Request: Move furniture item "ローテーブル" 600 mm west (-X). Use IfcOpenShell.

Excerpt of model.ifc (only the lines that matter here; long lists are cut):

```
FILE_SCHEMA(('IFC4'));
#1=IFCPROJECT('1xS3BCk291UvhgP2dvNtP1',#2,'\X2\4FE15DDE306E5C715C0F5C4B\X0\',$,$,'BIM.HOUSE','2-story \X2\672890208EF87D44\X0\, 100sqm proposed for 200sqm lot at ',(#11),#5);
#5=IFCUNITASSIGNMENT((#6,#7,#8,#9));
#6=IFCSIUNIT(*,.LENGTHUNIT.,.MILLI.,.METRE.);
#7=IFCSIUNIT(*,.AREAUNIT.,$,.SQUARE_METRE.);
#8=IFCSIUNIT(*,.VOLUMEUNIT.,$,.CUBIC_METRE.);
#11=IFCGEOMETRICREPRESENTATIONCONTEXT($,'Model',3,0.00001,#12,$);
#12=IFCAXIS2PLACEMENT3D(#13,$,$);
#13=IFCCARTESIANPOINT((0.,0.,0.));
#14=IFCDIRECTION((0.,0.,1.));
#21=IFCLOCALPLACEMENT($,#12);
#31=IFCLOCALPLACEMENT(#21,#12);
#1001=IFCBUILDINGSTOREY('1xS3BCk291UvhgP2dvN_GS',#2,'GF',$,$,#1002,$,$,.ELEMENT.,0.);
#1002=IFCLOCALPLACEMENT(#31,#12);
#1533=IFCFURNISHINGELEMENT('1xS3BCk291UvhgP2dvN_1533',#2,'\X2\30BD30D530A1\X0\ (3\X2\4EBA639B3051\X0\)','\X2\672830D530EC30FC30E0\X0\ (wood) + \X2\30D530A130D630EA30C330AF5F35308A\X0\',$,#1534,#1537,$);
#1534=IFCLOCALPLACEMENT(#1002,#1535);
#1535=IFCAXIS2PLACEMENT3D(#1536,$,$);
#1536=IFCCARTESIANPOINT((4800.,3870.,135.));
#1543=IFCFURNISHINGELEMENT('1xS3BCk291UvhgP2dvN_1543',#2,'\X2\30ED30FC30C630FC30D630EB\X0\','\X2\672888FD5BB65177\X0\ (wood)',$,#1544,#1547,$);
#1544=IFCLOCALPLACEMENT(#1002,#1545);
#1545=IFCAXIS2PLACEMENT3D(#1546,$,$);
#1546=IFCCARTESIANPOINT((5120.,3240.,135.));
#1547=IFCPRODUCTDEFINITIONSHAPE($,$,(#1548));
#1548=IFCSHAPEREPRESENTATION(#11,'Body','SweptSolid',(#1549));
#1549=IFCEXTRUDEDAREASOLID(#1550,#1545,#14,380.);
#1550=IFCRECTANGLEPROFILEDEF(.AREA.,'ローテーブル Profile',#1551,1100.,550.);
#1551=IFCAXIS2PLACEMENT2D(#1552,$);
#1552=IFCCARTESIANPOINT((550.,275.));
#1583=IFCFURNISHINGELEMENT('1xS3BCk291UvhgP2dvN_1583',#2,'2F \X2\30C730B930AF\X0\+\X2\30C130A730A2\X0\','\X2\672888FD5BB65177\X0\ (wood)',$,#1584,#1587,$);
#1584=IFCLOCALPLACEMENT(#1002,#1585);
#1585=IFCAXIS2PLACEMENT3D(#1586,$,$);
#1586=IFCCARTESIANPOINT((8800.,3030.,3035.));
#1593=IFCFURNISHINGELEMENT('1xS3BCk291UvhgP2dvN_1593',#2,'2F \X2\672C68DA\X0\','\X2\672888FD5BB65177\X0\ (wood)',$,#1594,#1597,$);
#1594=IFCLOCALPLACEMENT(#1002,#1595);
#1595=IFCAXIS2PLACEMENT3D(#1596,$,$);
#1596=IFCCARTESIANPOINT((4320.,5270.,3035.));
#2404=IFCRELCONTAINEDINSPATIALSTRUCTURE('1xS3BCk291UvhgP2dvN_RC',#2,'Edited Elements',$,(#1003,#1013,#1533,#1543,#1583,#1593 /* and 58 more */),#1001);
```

```python
import ifcopenshell
import ifcopenshell.api.geometry
import ifcopenshell.util.placement
import ifcopenshell.util.unit

model = ifcopenshell.open("model.ifc")
unit_scale = ifcopenshell.util.unit.calculate_unit_scale(model)

item = model.by_guid("1xS3BCk291UvhgP2dvN_1543")
matrix = ifcopenshell.util.placement.get_local_placement(item.ObjectPlacement)
matrix[0, 3] -= 0.6 / unit_scale
ifcopenshell.api.geometry.edit_object_placement(model, product=item, matrix=matrix, is_si=False)

print(ifcopenshell.util.placement.get_local_placement(item.ObjectPlacement).round(3) + 0.0)

model.write("model_updated.ifc")
```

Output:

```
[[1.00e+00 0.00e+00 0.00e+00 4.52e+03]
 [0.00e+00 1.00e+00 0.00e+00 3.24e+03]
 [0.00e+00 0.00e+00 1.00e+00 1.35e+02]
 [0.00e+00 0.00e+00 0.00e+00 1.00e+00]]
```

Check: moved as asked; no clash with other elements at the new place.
